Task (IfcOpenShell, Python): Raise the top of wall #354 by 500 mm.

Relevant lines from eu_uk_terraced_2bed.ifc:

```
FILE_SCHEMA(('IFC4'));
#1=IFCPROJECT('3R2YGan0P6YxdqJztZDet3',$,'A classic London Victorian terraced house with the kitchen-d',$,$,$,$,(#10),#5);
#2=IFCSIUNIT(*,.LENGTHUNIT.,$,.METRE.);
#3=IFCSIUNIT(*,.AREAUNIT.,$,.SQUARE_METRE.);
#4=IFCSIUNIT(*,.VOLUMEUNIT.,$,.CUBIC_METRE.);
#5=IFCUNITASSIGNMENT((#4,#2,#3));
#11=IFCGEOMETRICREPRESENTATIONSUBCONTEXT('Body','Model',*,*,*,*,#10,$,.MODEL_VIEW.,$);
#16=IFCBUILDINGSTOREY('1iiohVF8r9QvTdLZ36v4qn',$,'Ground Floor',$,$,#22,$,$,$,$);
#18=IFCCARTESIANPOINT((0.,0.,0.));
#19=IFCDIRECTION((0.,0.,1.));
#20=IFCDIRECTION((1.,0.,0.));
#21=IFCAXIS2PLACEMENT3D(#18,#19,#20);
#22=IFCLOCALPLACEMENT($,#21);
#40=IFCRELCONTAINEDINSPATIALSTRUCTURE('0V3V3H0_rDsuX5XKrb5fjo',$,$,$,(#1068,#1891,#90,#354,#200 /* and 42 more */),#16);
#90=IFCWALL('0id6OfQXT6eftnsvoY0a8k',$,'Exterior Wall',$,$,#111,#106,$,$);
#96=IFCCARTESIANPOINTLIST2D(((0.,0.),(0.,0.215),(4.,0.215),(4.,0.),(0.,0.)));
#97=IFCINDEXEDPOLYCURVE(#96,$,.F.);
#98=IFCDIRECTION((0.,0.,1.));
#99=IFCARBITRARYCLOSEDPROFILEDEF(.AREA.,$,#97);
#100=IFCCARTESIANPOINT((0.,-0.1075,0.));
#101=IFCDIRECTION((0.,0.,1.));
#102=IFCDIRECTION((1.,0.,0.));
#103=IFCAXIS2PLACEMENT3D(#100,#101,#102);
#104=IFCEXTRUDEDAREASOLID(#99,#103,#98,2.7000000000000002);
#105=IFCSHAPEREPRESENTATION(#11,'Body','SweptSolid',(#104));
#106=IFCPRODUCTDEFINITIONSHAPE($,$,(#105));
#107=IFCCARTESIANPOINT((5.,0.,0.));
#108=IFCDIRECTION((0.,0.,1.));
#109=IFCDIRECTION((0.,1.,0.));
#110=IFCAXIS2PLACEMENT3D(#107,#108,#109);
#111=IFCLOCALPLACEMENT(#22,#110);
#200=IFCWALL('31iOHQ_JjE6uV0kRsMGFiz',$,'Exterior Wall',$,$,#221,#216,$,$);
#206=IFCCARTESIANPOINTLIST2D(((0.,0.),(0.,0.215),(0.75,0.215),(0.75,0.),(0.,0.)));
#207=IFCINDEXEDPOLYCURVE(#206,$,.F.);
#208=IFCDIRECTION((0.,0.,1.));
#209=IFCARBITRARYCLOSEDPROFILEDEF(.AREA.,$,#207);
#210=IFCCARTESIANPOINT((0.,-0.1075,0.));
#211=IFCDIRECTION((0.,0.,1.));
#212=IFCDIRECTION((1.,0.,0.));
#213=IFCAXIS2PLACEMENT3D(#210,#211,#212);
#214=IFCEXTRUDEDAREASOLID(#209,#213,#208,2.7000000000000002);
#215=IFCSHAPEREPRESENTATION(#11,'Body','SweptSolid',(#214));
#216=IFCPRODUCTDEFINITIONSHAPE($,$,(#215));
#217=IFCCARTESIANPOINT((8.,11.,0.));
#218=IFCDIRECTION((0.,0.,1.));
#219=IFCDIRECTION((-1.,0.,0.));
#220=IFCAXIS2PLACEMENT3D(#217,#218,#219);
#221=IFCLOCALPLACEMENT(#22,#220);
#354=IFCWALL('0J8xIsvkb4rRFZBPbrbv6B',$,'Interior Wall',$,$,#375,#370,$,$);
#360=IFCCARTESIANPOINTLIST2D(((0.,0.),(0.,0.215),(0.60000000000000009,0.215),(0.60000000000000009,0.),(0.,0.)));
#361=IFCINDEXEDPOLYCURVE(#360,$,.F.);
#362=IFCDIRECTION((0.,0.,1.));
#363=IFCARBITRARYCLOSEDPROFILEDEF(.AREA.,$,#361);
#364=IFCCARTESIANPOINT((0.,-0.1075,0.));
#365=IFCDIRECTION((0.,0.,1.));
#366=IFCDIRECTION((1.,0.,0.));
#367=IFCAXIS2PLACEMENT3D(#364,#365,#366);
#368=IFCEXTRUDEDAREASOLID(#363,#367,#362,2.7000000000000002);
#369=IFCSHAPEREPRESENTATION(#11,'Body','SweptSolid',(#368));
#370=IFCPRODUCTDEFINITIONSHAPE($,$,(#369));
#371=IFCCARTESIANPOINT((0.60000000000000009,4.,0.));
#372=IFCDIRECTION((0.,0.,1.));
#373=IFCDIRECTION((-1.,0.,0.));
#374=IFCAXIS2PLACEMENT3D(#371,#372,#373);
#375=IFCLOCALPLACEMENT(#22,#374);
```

```python
import ifcopenshell
import ifcopenshell.geom
import ifcopenshell.util.representation
import ifcopenshell.util.shape
import ifcopenshell.util.unit

model = ifcopenshell.open("eu_uk_terraced_2bed.ifc")
unit_scale = ifcopenshell.util.unit.calculate_unit_scale(model)
settings = ifcopenshell.geom.settings()


def volume(element):
    """Net volume in cubic metres, openings subtracted."""
    shape = ifcopenshell.geom.create_shape(settings, element)
    return ifcopenshell.util.shape.get_volume(shape.geometry)


wall = model.by_id(354)
before = volume(wall)

body = ifcopenshell.util.representation.get_representation(wall, "Model", "Body")
solid = body.Items[0]
old_height = solid.Depth
solid.Depth += 0.5 / unit_scale
after = volume(wall)

print(f"height {old_height:g} -> {solid.Depth:g}, volume {before:.3f} -> {after:.3f} m3")

model.write("eu_uk_terraced_2bed_updated.ifc")
```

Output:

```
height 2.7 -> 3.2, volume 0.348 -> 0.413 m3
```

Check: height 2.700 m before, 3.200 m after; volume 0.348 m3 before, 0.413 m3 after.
